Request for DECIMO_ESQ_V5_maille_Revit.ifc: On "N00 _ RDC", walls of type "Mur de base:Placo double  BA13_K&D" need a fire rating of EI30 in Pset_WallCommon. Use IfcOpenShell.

First a look at what the model holds.

```python
import ifcopenshell
import ifcopenshell.util.element

model = ifcopenshell.open("DECIMO_ESQ_V5_maille_Revit.ifc")
print(model.schema)
storey = next(s for s in model.by_type("IfcBuildingStorey") if s.Name == "N00 _ RDC")
walls = [e for e in ifcopenshell.util.element.get_decomposition(storey) if e.is_a("IfcWall")]
seen = {}
for e in walls:
    element_type = ifcopenshell.util.element.get_type(e)
    key = (element_type.Name if element_type != e and element_type else None, ifcopenshell.util.element.get_pset(e, "Pset_WallCommon", "FireRating"))
    seen[key] = seen.get(key, 0) + 1
for (name, value), count in sorted(seen.items(), key=str):
    print(count, "x", name, "|", value)
```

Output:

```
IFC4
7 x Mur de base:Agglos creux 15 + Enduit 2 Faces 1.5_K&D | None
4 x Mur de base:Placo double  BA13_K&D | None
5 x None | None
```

```python
import ifcopenshell
import ifcopenshell.api.pset
import ifcopenshell.util.element

model = ifcopenshell.open("DECIMO_ESQ_V5_maille_Revit.ifc")

storey = next(s for s in model.by_type("IfcBuildingStorey") if s.Name == "N00 _ RDC")
walls = [e for e in ifcopenshell.util.element.get_decomposition(storey) if e.is_a("IfcWall")]

count = 0
for e in walls:
    element_type = ifcopenshell.util.element.get_type(e)
    if element_type in (None, e) or element_type.Name != "Mur de base:Placo double  BA13_K&D":
        continue
    # add_pset returns the element's existing set when there is one.
    pset = ifcopenshell.api.pset.add_pset(model, product=e, name="Pset_WallCommon")
    ifcopenshell.api.pset.edit_pset(model, pset=pset, properties={"FireRating": "EI30"})
    count += 1

print(count, "walls updated")

model.write("DECIMO_ESQ_V5_maille_Revit_rev.ifc")
```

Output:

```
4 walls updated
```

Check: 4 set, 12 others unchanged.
